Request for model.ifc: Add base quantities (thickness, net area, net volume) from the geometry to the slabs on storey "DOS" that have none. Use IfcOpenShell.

First a look at what the model holds.

```python
import ifcopenshell
import ifcopenshell.util.element
import ifcopenshell.util.unit

model = ifcopenshell.open("model.ifc")
print(model.schema)
for unit_type in ("LENGTHUNIT", "AREAUNIT", "VOLUMEUNIT"):
    print(unit_type, ifcopenshell.util.unit.calculate_unit_scale(model, unit_type))
storey = next(s for s in model.by_type("IfcBuildingStorey") if s.Name == "DOS")
slabs = [e for e in ifcopenshell.util.element.get_decomposition(storey) if e.is_a("IfcSlab")]
for e in sorted(slabs, key=lambda e: e.id()):
    print(e.id(), e.is_a(), e.Name, list(ifcopenshell.util.element.get_psets(e, qtos_only=True)), sep=" | ")
```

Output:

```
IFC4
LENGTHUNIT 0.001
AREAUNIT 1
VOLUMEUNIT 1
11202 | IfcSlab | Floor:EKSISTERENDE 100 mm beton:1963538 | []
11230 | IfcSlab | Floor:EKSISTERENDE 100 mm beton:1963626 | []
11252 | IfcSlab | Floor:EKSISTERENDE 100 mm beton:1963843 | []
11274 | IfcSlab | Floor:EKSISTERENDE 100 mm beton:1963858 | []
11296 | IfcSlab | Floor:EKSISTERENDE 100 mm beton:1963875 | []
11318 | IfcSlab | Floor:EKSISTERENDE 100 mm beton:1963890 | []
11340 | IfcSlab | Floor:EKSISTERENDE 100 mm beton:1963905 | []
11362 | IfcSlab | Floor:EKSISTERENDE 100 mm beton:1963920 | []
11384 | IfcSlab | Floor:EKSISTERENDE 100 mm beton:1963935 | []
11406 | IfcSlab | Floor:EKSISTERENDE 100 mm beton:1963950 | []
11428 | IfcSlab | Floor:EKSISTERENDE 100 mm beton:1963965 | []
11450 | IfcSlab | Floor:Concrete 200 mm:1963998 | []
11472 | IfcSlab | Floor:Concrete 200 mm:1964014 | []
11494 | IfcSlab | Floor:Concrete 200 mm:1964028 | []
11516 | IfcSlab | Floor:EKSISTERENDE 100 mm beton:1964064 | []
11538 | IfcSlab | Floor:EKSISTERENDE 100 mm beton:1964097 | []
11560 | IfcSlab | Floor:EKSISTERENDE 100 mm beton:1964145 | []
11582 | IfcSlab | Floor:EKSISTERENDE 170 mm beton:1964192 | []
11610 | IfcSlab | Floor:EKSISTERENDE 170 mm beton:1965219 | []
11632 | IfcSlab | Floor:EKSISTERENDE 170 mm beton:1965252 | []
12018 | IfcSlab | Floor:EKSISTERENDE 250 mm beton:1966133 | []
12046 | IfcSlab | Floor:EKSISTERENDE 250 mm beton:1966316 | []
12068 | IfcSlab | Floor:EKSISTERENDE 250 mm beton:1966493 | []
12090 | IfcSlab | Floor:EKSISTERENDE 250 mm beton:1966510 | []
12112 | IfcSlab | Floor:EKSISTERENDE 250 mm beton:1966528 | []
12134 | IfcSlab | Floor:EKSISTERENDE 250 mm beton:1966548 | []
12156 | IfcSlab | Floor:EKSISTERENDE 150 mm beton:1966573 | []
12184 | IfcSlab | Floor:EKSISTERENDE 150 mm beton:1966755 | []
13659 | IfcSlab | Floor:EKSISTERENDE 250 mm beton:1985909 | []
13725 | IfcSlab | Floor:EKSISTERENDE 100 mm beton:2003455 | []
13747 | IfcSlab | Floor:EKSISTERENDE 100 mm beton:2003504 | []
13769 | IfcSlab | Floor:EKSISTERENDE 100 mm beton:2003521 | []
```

```python
import ifcopenshell
import ifcopenshell.api.pset
import ifcopenshell.geom
import ifcopenshell.util.element
import ifcopenshell.util.shape
import ifcopenshell.util.unit

model = ifcopenshell.open("model.ifc")
unit_scale = ifcopenshell.util.unit.calculate_unit_scale(model)
area_scale = ifcopenshell.util.unit.calculate_unit_scale(model, "AREAUNIT")
volume_scale = ifcopenshell.util.unit.calculate_unit_scale(model, "VOLUMEUNIT")
settings = ifcopenshell.geom.settings()

storey = next(s for s in model.by_type("IfcBuildingStorey") if s.Name == "DOS")
slabs = [e for e in ifcopenshell.util.element.get_decomposition(storey) if e.is_a("IfcSlab")]

for e in sorted(slabs, key=lambda e: e.id()):
    if ifcopenshell.util.element.get_psets(e, qtos_only=True, should_inherit=False):
        continue
    # Geometry comes back in metres, in the element's own axes.
    shape = ifcopenshell.geom.create_shape(settings, e)
    values = {
        "Width": ifcopenshell.util.shape.get_z(shape.geometry) / unit_scale,
        "NetArea": ifcopenshell.util.shape.get_footprint_area(shape.geometry) / area_scale,
        "NetVolume": ifcopenshell.util.shape.get_volume(shape.geometry) / volume_scale,
    }
    qto = ifcopenshell.api.pset.add_qto(model, product=e, name="Qto_SlabBaseQuantities")
    ifcopenshell.api.pset.edit_qto(model, qto=qto, properties=values)
    print(e.id(), {k: round(v, 3) for k, v in values.items()})

model.write("model_v2.ifc")
```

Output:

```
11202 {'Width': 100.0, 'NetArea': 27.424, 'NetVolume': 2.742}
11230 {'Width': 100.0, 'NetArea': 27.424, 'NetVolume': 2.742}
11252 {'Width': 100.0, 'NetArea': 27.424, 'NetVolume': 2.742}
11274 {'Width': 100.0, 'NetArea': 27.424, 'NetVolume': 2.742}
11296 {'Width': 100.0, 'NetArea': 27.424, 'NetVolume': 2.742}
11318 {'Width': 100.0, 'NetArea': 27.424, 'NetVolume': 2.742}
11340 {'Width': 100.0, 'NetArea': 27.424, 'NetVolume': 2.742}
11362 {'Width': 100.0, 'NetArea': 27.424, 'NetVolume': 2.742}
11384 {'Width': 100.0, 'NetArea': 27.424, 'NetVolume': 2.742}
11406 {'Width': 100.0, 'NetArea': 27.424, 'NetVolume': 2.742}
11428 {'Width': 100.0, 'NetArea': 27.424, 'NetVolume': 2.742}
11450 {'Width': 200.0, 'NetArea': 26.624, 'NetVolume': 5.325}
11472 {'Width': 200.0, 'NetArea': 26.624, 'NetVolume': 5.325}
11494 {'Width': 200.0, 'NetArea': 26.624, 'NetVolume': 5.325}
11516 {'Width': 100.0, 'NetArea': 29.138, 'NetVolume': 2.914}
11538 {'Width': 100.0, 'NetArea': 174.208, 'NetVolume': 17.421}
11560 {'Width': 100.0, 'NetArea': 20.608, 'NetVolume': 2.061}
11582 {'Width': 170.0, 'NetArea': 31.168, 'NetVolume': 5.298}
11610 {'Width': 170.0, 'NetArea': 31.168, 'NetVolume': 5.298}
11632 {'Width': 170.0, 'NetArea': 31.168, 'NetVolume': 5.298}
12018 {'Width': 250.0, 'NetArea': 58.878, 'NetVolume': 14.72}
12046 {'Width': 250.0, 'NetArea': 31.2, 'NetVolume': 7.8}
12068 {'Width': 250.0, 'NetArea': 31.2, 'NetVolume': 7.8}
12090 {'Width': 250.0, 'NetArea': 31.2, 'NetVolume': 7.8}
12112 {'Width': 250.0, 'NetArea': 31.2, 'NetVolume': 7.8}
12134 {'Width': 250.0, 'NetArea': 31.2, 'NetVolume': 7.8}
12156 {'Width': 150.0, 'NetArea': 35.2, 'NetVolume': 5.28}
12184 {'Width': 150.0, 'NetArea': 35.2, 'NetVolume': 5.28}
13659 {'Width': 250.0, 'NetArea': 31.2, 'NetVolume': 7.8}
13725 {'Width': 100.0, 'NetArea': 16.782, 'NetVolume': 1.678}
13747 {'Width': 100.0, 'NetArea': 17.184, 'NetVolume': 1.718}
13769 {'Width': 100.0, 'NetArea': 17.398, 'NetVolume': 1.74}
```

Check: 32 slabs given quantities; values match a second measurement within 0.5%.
